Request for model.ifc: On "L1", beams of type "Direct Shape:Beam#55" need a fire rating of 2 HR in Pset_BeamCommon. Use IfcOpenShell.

First a look at what the model holds.

```python
import ifcopenshell
import ifcopenshell.util.element

model = ifcopenshell.open("model.ifc")
print(model.schema)
storey = next(s for s in model.by_type("IfcBuildingStorey") if s.Name == "L1")
beams = [e for e in ifcopenshell.util.element.get_decomposition(storey) if e.is_a("IfcBeam")]
seen = {}
for e in beams:
    element_type = ifcopenshell.util.element.get_type(e)
    key = (element_type.Name if element_type != e and element_type else None, ifcopenshell.util.element.get_pset(e, "Pset_BeamCommon", "FireRating"))
    seen[key] = seen.get(key, 0) + 1
for (name, value), count in sorted(seen.items(), key=str):
    print(count, "x", name, "|", value)
```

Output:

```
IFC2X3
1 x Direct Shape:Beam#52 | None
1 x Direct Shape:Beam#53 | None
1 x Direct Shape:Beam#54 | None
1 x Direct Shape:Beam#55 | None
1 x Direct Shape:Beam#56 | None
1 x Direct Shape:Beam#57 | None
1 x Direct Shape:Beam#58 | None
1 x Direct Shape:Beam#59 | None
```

```python
import ifcopenshell
import ifcopenshell.api.pset
import ifcopenshell.util.element

model = ifcopenshell.open("model.ifc")

storey = next(s for s in model.by_type("IfcBuildingStorey") if s.Name == "L1")
beams = [e for e in ifcopenshell.util.element.get_decomposition(storey) if e.is_a("IfcBeam")]

count = 0
for e in beams:
    element_type = ifcopenshell.util.element.get_type(e)
    if element_type in (None, e) or element_type.Name != "Direct Shape:Beam#55":
        continue
    # add_pset returns the element's existing set when there is one.
    pset = ifcopenshell.api.pset.add_pset(model, product=e, name="Pset_BeamCommon")
    ifcopenshell.api.pset.edit_pset(model, pset=pset, properties={"FireRating": "2 HR"})
    count += 1

print(count, "beams updated")

model.write("model_v2.ifc")
```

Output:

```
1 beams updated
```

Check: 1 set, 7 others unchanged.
